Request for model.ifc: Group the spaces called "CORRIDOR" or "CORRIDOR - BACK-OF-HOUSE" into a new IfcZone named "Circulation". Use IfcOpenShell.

First a look at what the model holds.

```python
import ifcopenshell

model = ifcopenshell.open("model.ifc")
print(model.schema)
seen = {}
for space in model.by_type("IfcSpace"):
    seen[space.LongName] = seen.get(space.LongName, 0) + 1
for name, count in sorted(seen.items(), key=str):
    print(count, "x", name)
print("zones:", [z.Name for z in model.by_type("IfcZone")][:20])
```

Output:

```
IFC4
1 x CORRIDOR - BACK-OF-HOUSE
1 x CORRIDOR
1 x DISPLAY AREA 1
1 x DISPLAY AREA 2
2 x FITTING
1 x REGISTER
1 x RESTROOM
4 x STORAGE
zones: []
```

```python
import ifcopenshell
import ifcopenshell.api.group
import ifcopenshell.api.root

model = ifcopenshell.open("model.ifc")

names = {"CORRIDOR", "CORRIDOR - BACK-OF-HOUSE"}
spaces = [s for s in model.by_type("IfcSpace") if s.LongName in names]

zone = ifcopenshell.api.root.create_entity(model, ifc_class="IfcZone", name="Circulation")
ifcopenshell.api.group.assign_group(model, products=spaces, group=zone)
print(len(spaces), "spaces in", zone.Name)

model.write("model_edited.ifc")
```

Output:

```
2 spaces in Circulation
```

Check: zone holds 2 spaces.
